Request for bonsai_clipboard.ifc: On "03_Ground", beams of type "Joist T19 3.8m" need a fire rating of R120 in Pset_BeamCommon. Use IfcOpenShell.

First a look at what the model holds.

```python
import ifcopenshell
import ifcopenshell.util.element

model = ifcopenshell.open("bonsai_clipboard.ifc")
print(model.schema)
storey = next(s for s in model.by_type("IfcBuildingStorey") if s.Name == "03_Ground")
beams = [e for e in ifcopenshell.util.element.get_decomposition(storey) if e.is_a("IfcBeam")]
seen = {}
for e in beams:
    element_type = ifcopenshell.util.element.get_type(e)
    key = (element_type.Name if element_type != e and element_type else None, ifcopenshell.util.element.get_pset(e, "Pset_BeamCommon", "FireRating"))
    seen[key] = seen.get(key, 0) + 1
for (name, value), count in sorted(seen.items(), key=str):
    print(count, "x", name, "|", value)
```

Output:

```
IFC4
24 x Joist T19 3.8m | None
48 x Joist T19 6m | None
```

```python
import ifcopenshell
import ifcopenshell.api.pset
import ifcopenshell.util.element

model = ifcopenshell.open("bonsai_clipboard.ifc")

storey = next(s for s in model.by_type("IfcBuildingStorey") if s.Name == "03_Ground")
beams = [e for e in ifcopenshell.util.element.get_decomposition(storey) if e.is_a("IfcBeam")]

count = 0
for e in beams:
    element_type = ifcopenshell.util.element.get_type(e)
    if element_type in (None, e) or element_type.Name != "Joist T19 3.8m":
        continue
    # add_pset returns the element's existing set when there is one.
    pset = ifcopenshell.api.pset.add_pset(model, product=e, name="Pset_BeamCommon")
    ifcopenshell.api.pset.edit_pset(model, pset=pset, properties={"FireRating": "R120"})
    count += 1

print(count, "beams updated")

model.write("bonsai_clipboard_updated.ifc")
```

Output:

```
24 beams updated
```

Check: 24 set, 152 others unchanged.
